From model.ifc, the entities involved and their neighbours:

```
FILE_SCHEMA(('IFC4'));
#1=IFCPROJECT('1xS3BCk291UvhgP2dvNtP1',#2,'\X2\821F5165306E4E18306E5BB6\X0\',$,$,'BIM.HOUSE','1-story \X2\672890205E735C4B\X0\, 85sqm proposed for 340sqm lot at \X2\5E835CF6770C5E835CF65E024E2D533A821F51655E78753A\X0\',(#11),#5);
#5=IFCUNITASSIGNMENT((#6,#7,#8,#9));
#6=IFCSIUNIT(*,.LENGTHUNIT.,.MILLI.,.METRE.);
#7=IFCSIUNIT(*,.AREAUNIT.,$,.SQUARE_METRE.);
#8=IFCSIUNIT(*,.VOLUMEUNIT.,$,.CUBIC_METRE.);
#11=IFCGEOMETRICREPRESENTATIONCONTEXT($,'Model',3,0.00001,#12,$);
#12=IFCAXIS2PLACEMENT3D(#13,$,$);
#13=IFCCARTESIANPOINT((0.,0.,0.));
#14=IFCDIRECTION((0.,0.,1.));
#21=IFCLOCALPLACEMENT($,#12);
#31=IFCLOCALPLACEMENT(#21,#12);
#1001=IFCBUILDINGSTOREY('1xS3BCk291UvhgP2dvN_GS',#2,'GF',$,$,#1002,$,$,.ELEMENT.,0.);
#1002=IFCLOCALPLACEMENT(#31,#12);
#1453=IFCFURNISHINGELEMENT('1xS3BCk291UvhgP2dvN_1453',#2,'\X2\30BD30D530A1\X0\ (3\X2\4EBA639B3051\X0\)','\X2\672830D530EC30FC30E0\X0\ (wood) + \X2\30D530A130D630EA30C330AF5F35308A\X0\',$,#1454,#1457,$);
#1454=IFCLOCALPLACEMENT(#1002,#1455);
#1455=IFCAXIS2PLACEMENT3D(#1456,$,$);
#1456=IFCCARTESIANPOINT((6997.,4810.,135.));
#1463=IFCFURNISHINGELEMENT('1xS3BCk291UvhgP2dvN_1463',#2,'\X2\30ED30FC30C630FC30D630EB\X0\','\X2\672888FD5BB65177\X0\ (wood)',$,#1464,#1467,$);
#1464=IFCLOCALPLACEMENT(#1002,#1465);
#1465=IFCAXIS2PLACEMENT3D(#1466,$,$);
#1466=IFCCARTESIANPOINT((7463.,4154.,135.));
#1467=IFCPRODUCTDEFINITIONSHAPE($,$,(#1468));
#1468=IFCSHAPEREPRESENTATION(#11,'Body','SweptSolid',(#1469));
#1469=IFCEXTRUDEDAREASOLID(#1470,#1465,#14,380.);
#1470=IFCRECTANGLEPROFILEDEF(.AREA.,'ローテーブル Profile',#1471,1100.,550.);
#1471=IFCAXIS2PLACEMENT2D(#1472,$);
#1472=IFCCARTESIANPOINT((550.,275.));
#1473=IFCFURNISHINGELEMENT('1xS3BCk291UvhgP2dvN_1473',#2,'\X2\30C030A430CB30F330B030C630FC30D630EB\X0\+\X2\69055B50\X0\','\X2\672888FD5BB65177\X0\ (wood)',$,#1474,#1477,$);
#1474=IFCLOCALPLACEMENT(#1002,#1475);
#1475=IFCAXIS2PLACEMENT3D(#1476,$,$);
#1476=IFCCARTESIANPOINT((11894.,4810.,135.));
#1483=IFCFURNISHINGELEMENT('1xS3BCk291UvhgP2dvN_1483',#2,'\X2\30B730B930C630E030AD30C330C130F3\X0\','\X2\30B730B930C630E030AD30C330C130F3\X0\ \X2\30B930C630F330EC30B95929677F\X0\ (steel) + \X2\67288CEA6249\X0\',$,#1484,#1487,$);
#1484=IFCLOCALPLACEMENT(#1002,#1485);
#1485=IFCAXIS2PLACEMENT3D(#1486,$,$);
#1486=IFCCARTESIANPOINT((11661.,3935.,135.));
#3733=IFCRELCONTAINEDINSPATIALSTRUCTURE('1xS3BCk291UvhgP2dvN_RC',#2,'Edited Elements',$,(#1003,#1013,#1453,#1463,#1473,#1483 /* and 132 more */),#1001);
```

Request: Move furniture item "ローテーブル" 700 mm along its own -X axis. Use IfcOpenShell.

```python
import ifcopenshell
import ifcopenshell.api.geometry
import ifcopenshell.util.placement
import ifcopenshell.util.unit

model = ifcopenshell.open("model.ifc")
unit_scale = ifcopenshell.util.unit.calculate_unit_scale(model)

item = model.by_guid("1xS3BCk291UvhgP2dvN_1463")
matrix = ifcopenshell.util.placement.get_local_placement(item.ObjectPlacement)
matrix[:3, 3] -= matrix[:3, 0] * 0.7 / unit_scale
ifcopenshell.api.geometry.edit_object_placement(model, product=item, matrix=matrix, is_si=False)

print(ifcopenshell.util.placement.get_local_placement(item.ObjectPlacement).round(3) + 0.0)

model.write("model_edited.ifc")
```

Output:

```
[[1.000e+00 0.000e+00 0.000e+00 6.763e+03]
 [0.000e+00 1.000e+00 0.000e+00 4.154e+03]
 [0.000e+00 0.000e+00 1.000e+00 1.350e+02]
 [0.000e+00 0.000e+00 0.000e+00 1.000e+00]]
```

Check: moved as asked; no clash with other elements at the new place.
